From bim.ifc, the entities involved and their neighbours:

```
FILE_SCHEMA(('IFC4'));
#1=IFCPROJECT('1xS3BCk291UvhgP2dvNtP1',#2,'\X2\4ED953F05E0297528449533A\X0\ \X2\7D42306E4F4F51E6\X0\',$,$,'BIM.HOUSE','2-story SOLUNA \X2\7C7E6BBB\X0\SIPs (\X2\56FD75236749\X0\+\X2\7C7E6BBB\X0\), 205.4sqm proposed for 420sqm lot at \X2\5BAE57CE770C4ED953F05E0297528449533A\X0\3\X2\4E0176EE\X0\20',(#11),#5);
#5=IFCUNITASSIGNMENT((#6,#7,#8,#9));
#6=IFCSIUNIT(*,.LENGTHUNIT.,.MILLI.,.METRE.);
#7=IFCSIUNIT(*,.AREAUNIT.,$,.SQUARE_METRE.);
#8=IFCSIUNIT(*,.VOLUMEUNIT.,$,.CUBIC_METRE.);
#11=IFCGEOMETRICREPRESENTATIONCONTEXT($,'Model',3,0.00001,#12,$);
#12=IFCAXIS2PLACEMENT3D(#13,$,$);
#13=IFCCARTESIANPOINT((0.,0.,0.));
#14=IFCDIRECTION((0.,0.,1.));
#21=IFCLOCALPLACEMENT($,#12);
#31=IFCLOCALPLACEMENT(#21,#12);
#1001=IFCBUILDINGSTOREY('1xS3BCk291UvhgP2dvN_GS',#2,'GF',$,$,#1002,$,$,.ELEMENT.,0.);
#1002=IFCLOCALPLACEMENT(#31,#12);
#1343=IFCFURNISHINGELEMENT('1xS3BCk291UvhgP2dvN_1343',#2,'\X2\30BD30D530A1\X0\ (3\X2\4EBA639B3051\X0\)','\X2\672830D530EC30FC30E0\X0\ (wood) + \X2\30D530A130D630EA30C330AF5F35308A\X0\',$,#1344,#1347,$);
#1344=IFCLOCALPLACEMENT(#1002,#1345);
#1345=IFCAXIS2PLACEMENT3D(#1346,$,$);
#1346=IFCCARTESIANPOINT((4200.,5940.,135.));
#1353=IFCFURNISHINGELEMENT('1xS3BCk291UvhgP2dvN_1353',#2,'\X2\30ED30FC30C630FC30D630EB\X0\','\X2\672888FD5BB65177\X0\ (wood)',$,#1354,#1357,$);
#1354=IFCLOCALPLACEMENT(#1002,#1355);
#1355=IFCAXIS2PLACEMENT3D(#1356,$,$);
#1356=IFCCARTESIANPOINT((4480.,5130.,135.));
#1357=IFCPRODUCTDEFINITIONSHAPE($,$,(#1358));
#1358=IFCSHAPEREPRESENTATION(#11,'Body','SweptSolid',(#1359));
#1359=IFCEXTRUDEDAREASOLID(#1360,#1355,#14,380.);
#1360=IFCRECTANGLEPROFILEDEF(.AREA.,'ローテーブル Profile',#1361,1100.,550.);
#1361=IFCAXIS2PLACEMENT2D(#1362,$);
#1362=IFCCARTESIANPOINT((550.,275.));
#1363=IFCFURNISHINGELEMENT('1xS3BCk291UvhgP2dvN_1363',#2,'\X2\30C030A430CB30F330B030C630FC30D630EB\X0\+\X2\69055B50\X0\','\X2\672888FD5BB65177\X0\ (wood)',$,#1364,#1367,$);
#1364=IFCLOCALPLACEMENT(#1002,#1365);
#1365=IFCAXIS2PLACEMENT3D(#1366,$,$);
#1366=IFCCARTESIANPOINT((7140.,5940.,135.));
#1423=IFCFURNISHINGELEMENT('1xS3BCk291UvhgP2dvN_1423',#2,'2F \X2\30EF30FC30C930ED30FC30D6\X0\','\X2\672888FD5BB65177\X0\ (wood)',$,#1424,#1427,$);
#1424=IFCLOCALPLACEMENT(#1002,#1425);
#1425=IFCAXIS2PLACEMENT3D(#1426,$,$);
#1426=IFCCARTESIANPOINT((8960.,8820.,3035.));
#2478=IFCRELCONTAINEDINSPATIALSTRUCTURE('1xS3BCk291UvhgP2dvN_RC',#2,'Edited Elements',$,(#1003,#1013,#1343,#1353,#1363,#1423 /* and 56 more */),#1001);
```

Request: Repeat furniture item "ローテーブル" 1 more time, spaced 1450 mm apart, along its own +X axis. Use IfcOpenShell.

```python
import ifcopenshell
import ifcopenshell.api.geometry
import ifcopenshell.api.root
import ifcopenshell.util.element
import ifcopenshell.util.placement

model = ifcopenshell.open("bim.ifc")


def reuse_history(source, copy):
    """copy_class also copies each property set's owner history, people and application; keep the originals."""
    for rel in copy.IsDefinedBy:
        if rel.is_a("IfcRelDefinesByProperties") and (history := rel.RelatingPropertyDefinition.OwnerHistory):
            rel.RelatingPropertyDefinition.OwnerHistory = source.OwnerHistory
            ifcopenshell.util.element.remove_deep2(model, history)


source = model.by_guid("1xS3BCk291UvhgP2dvN_1353")
base = ifcopenshell.util.placement.get_local_placement(source.ObjectPlacement)
step = base[:3, 0] * 1450.0

for i in range(1, 2):
    copy = ifcopenshell.api.root.copy_class(model, product=source)
    copy.Representation = ifcopenshell.util.element.copy_deep(
        model, source.Representation, exclude=["IfcGeometricRepresentationContext", "IfcRepresentationMap"]
    )
    reuse_history(source, copy)
    matrix = base.copy()
    matrix[:3, 3] += i * step
    print("added at", matrix[:3, 3].round(3) + 0.0)
    ifcopenshell.api.geometry.edit_object_placement(model, product=copy, matrix=matrix, is_si=False)

model.write("bim_edited.ifc")
```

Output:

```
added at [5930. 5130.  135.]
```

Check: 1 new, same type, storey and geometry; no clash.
